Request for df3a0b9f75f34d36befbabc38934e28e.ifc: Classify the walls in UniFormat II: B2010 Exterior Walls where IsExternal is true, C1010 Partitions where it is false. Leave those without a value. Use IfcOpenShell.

First a look at what the model holds.

```python
import ifcopenshell
import ifcopenshell.util.element

model = ifcopenshell.open("df3a0b9f75f34d36befbabc38934e28e.ifc")
print(model.schema)
print("classifications:", [c.Name for c in model.by_type("IfcClassification")])
values = [ifcopenshell.util.element.get_pset(e, "Pset_WallCommon", "IsExternal") for e in model.by_type("IfcWall")]
for value in (True, False, None):
    print("IsExternal", value, values.count(value))
```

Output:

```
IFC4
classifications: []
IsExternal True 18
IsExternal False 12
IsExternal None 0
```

```python
import ifcopenshell
import ifcopenshell.api.classification
import ifcopenshell.util.element

model = ifcopenshell.open("df3a0b9f75f34d36befbabc38934e28e.ifc")

system = ifcopenshell.api.classification.add_classification(model, classification="UniFormat II")

walls = model.by_type("IfcWall")
external = {e: ifcopenshell.util.element.get_pset(e, "Pset_WallCommon", "IsExternal") for e in walls}
for flag, code, name in ((True, "B2010", "Exterior Walls"), (False, "C1010", "Partitions")):
    products = [e for e in walls if external[e] is flag]
    ifcopenshell.api.classification.add_reference(
        model, products=products, classification=system, identification=code, name=name
    )
    print(code, len(products))

model.write("df3a0b9f75f34d36befbabc38934e28e_rev.ifc")
```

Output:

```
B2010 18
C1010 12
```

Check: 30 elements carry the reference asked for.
